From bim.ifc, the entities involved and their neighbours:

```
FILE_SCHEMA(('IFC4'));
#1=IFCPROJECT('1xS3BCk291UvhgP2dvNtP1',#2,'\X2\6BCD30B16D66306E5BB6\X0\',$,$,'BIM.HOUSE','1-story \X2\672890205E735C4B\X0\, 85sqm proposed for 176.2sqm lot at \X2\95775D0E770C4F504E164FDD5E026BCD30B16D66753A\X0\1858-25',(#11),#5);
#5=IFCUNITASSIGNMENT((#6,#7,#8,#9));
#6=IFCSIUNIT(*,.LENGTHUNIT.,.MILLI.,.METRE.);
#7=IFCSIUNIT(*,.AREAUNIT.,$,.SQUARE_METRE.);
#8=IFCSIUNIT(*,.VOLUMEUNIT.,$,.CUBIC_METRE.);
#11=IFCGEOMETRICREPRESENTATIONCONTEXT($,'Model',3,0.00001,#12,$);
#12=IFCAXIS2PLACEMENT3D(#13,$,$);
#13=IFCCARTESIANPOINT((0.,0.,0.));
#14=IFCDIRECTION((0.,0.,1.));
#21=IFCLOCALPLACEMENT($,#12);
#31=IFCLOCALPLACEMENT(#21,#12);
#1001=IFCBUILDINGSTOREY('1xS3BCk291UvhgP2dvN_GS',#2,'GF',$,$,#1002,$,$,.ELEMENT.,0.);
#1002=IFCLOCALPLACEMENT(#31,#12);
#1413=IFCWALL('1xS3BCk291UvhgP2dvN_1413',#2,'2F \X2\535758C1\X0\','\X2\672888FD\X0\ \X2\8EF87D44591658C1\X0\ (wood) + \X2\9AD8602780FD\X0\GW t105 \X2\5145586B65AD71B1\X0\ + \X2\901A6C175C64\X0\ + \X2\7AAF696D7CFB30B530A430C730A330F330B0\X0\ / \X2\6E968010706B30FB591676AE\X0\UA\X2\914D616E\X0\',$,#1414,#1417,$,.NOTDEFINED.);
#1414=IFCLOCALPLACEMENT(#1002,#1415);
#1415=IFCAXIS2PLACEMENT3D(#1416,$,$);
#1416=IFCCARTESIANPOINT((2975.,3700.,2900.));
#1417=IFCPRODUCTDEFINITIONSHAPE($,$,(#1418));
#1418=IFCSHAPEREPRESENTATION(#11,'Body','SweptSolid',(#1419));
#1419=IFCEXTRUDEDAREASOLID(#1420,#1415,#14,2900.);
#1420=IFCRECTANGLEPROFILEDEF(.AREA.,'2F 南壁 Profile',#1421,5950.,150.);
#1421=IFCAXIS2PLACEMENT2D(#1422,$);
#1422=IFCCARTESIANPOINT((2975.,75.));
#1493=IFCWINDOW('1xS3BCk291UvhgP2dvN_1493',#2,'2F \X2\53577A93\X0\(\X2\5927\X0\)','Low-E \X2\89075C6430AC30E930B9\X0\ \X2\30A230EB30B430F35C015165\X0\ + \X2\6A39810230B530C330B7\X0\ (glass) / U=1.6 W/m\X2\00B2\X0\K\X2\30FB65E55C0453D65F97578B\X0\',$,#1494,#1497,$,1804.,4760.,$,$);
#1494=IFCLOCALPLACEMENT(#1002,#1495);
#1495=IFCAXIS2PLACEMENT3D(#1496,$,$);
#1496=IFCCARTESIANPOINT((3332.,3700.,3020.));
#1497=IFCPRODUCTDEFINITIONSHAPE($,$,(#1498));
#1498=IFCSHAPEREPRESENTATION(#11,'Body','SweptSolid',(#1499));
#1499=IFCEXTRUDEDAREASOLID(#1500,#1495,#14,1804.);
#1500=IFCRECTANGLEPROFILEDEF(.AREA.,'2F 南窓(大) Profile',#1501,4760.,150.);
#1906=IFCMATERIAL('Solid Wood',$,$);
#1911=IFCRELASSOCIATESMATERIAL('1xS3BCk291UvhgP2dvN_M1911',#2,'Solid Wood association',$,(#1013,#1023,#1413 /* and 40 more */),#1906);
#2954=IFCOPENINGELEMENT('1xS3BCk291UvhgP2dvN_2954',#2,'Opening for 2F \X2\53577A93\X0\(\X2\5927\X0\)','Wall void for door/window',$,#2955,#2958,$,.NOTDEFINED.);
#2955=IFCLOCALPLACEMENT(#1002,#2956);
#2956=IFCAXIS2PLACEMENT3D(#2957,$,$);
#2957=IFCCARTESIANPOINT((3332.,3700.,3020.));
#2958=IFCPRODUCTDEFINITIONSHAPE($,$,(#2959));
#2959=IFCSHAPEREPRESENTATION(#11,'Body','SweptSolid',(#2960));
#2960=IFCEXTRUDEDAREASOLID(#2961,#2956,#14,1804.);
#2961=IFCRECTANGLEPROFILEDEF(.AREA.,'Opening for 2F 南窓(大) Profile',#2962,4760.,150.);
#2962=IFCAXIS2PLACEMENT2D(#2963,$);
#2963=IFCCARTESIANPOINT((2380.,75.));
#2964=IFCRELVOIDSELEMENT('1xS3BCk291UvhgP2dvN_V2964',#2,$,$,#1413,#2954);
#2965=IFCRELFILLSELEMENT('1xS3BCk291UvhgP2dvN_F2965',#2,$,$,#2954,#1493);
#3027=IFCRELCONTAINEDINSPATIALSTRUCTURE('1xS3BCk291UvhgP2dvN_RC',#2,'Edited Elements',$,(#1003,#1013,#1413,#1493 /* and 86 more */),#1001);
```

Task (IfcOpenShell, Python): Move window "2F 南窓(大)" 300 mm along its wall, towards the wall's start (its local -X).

```python
import ifcopenshell
import ifcopenshell.api.geometry
import ifcopenshell.util.placement
import ifcopenshell.util.unit

model = ifcopenshell.open("bim.ifc")
unit_scale = ifcopenshell.util.unit.calculate_unit_scale(model)

window = model.by_guid("1xS3BCk291UvhgP2dvN_1493")
opening = window.FillsVoids[0].RelatingOpeningElement
wall = opening.VoidsElements[0].RelatingBuildingElement

wall_matrix = ifcopenshell.util.placement.get_local_placement(wall.ObjectPlacement)
shift = wall_matrix[:3, 0] * -0.3 / unit_scale
before = ifcopenshell.util.placement.get_local_placement(window.ObjectPlacement)[:3, 3].copy()

# The window is not placed relative to its opening, so move both.
for product in (opening, window):
    matrix = ifcopenshell.util.placement.get_local_placement(product.ObjectPlacement)
    matrix[:3, 3] += shift
    ifcopenshell.api.geometry.edit_object_placement(model, product=product, matrix=matrix, is_si=False)

after = ifcopenshell.util.placement.get_local_placement(window.ObjectPlacement)[:3, 3]
print("window moved by", (after - before).round(3) + 0.0)

model.write("bim_rev.ifc")
```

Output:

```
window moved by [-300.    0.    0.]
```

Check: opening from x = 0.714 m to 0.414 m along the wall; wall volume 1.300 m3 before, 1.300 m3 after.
